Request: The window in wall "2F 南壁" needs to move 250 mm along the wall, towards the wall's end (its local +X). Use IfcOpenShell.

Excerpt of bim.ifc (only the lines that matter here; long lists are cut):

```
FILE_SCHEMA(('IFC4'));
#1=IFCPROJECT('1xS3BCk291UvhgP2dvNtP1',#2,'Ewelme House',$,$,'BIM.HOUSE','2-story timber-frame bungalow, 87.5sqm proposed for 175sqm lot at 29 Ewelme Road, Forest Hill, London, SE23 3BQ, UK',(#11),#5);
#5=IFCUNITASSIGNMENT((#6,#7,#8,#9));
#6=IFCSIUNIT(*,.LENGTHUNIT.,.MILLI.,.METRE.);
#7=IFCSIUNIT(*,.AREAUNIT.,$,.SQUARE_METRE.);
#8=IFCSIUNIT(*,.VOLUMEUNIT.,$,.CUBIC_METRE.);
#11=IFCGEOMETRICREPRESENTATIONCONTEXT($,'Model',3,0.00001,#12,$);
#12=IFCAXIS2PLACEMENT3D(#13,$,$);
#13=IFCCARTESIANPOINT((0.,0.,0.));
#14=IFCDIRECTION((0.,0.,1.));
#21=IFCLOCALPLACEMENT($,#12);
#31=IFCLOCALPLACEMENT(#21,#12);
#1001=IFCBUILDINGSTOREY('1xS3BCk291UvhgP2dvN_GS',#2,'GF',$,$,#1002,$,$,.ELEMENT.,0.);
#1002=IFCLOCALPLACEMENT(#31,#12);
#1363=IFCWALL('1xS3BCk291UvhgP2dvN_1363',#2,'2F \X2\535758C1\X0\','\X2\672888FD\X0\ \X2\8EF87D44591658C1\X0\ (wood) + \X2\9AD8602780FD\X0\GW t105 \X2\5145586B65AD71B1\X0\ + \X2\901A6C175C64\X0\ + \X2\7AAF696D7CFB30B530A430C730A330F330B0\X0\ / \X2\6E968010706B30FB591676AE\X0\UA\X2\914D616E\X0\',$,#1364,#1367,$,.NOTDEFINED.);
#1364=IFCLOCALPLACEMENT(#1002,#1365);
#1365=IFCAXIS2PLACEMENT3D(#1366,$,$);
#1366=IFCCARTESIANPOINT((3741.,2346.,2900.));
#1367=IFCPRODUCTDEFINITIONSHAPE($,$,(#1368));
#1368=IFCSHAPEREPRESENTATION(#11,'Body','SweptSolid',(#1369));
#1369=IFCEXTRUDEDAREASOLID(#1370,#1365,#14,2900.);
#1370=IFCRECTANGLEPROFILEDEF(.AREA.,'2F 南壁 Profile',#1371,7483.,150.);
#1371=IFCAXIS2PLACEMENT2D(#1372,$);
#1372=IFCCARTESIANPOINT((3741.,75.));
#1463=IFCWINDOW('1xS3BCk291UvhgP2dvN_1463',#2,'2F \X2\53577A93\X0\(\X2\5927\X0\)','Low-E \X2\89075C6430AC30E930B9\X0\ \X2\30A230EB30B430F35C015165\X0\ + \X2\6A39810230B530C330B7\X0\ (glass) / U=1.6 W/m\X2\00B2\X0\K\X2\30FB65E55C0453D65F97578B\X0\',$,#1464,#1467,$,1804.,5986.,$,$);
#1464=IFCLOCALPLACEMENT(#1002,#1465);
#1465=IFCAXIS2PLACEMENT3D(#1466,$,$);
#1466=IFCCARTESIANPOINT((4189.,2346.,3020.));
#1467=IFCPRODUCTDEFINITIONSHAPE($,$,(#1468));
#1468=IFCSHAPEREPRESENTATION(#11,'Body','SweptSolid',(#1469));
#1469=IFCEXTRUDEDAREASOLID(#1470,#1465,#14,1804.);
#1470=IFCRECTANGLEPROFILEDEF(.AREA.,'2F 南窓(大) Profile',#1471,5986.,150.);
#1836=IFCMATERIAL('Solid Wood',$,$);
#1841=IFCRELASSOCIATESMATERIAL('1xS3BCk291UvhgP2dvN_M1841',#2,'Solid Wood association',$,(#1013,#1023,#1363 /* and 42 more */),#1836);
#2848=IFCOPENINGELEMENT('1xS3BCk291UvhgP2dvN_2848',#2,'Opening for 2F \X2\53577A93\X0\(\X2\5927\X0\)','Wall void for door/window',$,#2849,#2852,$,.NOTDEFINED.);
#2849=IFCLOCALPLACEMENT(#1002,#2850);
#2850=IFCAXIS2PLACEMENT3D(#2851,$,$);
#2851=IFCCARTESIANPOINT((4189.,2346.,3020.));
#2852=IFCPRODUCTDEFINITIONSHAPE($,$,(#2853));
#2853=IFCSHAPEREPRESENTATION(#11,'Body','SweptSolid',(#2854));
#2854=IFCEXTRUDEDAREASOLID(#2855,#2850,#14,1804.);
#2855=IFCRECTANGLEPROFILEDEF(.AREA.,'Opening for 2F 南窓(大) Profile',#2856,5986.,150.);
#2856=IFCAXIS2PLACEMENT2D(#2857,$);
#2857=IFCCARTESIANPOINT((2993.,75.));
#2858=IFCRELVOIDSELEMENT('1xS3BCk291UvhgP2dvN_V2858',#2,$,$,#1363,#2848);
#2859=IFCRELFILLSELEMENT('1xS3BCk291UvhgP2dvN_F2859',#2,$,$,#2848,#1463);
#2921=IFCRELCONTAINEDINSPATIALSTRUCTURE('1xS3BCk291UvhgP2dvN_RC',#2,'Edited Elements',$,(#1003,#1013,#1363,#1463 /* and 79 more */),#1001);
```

```python
import ifcopenshell
import ifcopenshell.api.geometry
import ifcopenshell.util.placement
import ifcopenshell.util.unit

model = ifcopenshell.open("bim.ifc")
unit_scale = ifcopenshell.util.unit.calculate_unit_scale(model)

window = model.by_guid("1xS3BCk291UvhgP2dvN_1463")
opening = window.FillsVoids[0].RelatingOpeningElement
wall = opening.VoidsElements[0].RelatingBuildingElement

wall_matrix = ifcopenshell.util.placement.get_local_placement(wall.ObjectPlacement)
shift = wall_matrix[:3, 0] * 0.25 / unit_scale
before = ifcopenshell.util.placement.get_local_placement(window.ObjectPlacement)[:3, 3].copy()

# The window is not placed relative to its opening, so move both.
for product in (opening, window):
    matrix = ifcopenshell.util.placement.get_local_placement(product.ObjectPlacement)
    matrix[:3, 3] += shift
    ifcopenshell.api.geometry.edit_object_placement(model, product=product, matrix=matrix, is_si=False)

after = ifcopenshell.util.placement.get_local_placement(window.ObjectPlacement)[:3, 3]
print("window moved by", (after - before).round(3) + 0.0)

model.write("bim_rev.ifc")
```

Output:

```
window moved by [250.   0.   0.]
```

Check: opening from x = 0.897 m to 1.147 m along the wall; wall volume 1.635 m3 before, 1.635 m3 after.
